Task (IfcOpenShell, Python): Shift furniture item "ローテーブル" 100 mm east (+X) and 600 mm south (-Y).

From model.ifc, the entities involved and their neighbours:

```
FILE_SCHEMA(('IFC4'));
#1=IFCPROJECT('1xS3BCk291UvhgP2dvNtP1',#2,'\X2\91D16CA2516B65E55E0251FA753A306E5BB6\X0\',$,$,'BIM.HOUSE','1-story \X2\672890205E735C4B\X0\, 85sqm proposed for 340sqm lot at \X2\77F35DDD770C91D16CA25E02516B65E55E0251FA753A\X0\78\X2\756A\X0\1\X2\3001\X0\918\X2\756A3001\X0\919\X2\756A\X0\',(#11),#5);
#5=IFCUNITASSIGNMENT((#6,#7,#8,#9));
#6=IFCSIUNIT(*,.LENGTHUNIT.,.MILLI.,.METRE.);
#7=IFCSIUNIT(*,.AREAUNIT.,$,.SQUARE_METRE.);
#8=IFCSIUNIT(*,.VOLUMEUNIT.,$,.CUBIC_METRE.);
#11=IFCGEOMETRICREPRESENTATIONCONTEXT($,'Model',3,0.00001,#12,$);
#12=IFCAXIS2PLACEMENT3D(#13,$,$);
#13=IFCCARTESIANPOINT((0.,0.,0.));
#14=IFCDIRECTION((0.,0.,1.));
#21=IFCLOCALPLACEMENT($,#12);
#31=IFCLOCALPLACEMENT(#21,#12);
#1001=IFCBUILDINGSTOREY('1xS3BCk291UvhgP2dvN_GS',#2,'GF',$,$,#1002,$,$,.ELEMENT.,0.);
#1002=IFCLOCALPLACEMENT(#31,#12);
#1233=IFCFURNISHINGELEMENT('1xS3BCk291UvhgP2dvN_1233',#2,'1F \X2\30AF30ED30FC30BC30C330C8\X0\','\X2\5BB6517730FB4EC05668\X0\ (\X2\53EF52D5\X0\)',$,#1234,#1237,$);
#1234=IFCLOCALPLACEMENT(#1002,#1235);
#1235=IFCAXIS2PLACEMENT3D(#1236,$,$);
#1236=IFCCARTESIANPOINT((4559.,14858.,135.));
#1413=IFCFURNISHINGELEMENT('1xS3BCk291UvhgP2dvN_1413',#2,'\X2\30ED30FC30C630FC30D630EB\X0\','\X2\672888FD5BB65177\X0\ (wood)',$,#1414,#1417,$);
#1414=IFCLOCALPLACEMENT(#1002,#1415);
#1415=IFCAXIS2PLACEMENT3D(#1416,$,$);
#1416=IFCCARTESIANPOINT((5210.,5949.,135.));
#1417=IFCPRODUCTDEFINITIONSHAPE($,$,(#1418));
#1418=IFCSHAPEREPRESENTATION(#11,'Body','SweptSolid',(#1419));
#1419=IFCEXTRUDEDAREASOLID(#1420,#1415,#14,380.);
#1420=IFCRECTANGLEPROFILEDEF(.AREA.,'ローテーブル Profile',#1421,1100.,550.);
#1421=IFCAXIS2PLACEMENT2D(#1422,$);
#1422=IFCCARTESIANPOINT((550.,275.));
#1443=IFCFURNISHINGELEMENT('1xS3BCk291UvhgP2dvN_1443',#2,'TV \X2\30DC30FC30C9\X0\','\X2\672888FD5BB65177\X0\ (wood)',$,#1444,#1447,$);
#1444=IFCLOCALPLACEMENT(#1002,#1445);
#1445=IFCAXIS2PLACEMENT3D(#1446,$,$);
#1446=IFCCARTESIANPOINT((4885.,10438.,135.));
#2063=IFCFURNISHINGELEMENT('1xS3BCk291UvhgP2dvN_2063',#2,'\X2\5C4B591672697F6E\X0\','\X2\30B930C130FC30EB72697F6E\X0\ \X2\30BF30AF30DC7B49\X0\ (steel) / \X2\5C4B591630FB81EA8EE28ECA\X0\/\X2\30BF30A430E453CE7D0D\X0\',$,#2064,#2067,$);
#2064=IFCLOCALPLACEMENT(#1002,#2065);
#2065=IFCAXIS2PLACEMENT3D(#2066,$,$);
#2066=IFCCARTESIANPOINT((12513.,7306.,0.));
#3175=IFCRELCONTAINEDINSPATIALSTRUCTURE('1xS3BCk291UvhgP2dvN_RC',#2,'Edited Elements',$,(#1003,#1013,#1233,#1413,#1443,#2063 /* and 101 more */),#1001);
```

```python
import ifcopenshell
import ifcopenshell.api.geometry
import ifcopenshell.util.placement

model = ifcopenshell.open("model.ifc")

item = model.by_id(1413)
matrix = ifcopenshell.util.placement.get_local_placement(item.ObjectPlacement)
matrix[0, 3] += 100.0
matrix[1, 3] -= 600.0
ifcopenshell.api.geometry.edit_object_placement(model, product=item, matrix=matrix, is_si=False)

print(ifcopenshell.util.placement.get_local_placement(item.ObjectPlacement).round(3) + 0.0)

model.write("model_v2.ifc")
```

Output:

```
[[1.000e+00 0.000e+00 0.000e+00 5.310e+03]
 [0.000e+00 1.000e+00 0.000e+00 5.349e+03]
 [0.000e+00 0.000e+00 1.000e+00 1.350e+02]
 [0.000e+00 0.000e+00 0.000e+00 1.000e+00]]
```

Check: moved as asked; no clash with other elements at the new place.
